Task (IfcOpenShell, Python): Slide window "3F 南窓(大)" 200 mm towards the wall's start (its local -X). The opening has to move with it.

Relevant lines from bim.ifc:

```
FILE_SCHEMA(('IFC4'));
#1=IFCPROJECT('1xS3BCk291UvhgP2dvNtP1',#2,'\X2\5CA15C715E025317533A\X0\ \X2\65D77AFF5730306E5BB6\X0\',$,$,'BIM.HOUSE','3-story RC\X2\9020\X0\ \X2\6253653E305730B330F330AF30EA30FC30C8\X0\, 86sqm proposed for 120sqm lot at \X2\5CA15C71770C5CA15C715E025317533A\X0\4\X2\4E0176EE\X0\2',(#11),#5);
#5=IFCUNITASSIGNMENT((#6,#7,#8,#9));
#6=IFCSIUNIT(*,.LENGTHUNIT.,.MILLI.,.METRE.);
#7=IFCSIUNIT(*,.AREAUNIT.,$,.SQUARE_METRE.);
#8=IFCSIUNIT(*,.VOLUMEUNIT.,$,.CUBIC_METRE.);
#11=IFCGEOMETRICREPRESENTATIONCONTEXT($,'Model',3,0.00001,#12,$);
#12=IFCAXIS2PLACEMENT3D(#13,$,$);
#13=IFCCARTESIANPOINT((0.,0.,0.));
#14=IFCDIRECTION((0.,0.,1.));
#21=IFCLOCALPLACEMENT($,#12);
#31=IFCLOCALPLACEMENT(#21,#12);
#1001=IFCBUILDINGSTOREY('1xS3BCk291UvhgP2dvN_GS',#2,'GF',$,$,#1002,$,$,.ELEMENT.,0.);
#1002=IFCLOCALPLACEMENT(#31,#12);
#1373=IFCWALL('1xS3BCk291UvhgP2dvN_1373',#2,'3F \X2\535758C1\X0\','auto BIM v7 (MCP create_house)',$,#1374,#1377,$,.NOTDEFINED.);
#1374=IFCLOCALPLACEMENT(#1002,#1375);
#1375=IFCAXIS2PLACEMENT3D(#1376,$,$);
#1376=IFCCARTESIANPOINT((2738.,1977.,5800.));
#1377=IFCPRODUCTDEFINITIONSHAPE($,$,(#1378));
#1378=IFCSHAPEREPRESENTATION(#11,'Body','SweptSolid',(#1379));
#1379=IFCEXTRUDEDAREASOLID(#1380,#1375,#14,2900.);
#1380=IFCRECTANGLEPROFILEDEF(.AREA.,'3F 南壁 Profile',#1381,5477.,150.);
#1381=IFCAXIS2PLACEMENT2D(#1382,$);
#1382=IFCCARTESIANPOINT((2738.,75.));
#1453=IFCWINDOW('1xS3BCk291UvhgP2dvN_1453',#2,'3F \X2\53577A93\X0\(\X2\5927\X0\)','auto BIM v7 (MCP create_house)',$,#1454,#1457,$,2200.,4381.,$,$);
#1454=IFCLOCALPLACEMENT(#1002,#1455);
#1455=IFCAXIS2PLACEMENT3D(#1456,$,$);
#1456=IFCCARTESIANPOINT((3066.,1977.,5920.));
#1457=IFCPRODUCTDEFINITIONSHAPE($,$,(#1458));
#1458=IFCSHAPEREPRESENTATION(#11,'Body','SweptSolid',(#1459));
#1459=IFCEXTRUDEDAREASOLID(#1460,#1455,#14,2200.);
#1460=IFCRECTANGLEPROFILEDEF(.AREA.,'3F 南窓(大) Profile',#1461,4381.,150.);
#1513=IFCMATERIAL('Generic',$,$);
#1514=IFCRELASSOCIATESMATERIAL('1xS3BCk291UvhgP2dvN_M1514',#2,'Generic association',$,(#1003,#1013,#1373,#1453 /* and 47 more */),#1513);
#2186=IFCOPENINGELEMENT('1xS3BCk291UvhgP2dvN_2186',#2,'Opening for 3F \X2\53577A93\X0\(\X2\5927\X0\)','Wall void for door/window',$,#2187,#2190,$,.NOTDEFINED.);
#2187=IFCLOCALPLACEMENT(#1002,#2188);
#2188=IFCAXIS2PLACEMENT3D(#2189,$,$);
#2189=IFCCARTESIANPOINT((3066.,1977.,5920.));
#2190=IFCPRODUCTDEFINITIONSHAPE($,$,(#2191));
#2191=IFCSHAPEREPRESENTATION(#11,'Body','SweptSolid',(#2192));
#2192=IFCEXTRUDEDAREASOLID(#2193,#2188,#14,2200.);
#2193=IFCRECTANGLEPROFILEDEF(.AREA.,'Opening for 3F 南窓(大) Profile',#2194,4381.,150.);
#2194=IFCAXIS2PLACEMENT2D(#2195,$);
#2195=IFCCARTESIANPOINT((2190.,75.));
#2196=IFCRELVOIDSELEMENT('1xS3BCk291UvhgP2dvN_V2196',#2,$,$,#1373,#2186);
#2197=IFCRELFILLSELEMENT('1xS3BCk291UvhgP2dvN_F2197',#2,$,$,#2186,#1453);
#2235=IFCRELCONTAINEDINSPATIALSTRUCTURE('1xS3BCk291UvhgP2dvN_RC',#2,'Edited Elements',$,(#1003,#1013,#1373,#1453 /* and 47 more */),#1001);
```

```python
import ifcopenshell
import ifcopenshell.api.geometry
import ifcopenshell.util.placement

model = ifcopenshell.open("bim.ifc")

window = model.by_guid("1xS3BCk291UvhgP2dvN_1453")
opening = window.FillsVoids[0].RelatingOpeningElement
wall = opening.VoidsElements[0].RelatingBuildingElement

wall_matrix = ifcopenshell.util.placement.get_local_placement(wall.ObjectPlacement)
shift = wall_matrix[:3, 0] * -200.0
before = ifcopenshell.util.placement.get_local_placement(window.ObjectPlacement)[:3, 3].copy()

# The window is not placed relative to its opening, so move both.
for product in (opening, window):
    matrix = ifcopenshell.util.placement.get_local_placement(product.ObjectPlacement)
    matrix[:3, 3] += shift
    ifcopenshell.api.geometry.edit_object_placement(model, product=product, matrix=matrix, is_si=False)

after = ifcopenshell.util.placement.get_local_placement(window.ObjectPlacement)[:3, 3]
print("window moved by", (after - before).round(3) + 0.0)

model.write("bim_v2.ifc")
```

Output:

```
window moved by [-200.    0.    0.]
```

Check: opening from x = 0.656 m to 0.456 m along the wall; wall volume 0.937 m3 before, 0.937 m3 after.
